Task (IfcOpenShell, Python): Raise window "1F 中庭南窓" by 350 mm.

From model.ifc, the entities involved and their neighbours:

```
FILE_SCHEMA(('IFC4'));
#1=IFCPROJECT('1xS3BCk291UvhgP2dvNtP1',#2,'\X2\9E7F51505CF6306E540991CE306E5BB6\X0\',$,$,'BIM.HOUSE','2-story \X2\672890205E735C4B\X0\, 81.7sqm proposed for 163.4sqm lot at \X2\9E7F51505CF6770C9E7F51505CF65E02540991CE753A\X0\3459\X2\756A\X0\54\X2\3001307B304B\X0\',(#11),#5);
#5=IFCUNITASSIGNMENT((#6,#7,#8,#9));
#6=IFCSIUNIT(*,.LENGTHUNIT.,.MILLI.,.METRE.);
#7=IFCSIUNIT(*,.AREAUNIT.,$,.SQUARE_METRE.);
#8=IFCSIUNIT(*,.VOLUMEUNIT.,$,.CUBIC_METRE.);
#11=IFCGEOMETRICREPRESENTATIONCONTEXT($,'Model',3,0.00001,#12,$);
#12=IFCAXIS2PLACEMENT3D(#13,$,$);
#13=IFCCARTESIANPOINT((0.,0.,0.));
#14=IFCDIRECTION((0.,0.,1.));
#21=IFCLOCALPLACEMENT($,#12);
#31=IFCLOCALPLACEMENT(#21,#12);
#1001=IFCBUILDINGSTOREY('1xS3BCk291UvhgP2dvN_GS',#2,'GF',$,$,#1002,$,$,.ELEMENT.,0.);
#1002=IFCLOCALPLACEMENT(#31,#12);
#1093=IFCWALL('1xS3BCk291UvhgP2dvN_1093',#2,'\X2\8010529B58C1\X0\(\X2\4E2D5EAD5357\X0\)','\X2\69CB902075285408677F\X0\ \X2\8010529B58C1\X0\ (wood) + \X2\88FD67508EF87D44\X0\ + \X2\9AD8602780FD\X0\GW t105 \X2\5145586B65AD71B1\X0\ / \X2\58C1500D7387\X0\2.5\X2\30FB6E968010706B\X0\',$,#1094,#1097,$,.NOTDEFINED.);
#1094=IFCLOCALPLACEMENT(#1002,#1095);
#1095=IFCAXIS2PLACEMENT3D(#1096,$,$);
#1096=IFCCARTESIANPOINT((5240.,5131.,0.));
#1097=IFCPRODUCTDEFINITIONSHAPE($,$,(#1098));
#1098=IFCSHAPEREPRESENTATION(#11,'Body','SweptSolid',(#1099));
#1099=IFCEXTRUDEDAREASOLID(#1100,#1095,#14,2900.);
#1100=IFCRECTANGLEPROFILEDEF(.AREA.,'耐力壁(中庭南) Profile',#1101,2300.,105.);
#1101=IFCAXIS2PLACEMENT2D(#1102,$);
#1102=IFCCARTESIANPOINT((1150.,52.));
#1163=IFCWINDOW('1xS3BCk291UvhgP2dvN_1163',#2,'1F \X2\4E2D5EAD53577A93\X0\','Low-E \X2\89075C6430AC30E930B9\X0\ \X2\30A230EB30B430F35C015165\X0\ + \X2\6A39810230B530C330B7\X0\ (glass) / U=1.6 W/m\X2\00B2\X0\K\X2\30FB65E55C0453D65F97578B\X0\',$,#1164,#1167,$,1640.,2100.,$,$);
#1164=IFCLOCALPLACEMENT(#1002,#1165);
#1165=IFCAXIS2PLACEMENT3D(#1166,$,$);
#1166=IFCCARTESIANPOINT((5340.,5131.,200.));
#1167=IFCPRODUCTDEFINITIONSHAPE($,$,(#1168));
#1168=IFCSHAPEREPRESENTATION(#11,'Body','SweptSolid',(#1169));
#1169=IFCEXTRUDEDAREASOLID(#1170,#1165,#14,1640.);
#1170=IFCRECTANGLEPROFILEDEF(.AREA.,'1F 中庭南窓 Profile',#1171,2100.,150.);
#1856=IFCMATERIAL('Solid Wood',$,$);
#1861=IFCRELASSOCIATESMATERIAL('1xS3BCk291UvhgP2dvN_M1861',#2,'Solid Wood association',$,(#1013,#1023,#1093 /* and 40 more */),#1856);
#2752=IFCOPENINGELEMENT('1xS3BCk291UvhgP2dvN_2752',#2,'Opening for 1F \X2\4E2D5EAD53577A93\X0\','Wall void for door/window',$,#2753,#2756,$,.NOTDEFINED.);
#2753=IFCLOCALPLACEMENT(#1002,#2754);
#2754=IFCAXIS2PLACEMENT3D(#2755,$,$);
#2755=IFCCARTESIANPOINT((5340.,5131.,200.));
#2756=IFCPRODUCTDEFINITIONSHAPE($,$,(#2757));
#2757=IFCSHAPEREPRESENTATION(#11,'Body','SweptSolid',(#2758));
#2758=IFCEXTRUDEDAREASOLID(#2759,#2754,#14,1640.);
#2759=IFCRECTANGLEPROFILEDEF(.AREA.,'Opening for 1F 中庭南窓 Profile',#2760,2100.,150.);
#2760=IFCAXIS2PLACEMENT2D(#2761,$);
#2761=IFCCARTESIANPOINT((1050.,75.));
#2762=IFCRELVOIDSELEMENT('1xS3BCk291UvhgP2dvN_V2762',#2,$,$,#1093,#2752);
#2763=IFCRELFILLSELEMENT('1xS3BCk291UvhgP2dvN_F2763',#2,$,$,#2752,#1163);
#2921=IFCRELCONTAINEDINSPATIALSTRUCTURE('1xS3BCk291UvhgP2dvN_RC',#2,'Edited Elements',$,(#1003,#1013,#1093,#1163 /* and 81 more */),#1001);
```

```python
import numpy as np
import ifcopenshell
import ifcopenshell.api.geometry
import ifcopenshell.util.placement
import ifcopenshell.util.unit

model = ifcopenshell.open("model.ifc")
unit_scale = ifcopenshell.util.unit.calculate_unit_scale(model)

window = model.by_id(1163)
opening = window.FillsVoids[0].RelatingOpeningElement
dz = 0.35 / unit_scale

shift = np.array([0.0, 0.0, dz])
# The window is not placed relative to its opening, so move both.
for product in (opening, window):
    matrix = ifcopenshell.util.placement.get_local_placement(product.ObjectPlacement)
    matrix[:3, 3] += shift
    ifcopenshell.api.geometry.edit_object_placement(model, product=product, matrix=matrix, is_si=False)

print(f"moved by {dz * unit_scale:+.3f} m")

model.write("model-out.ifc")
```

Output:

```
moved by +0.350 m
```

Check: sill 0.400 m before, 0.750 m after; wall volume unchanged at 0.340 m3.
